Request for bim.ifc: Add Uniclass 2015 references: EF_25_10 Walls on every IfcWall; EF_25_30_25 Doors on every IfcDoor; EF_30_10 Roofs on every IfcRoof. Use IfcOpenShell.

First a look at what the model holds.

```python
import ifcopenshell

model = ifcopenshell.open("bim.ifc")
print(model.schema)
print("classifications:", [c.Name for c in model.by_type("IfcClassification")])
for ifc_class in ("IfcDoor", "IfcRoof", "IfcStair", "IfcWall", "IfcWindow"):
    print(ifc_class, len(model.by_type(ifc_class)))
```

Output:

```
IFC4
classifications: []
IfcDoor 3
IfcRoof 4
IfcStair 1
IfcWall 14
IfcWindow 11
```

```python
import ifcopenshell
import ifcopenshell.api.classification

model = ifcopenshell.open("bim.ifc")

system = ifcopenshell.api.classification.add_classification(model, classification="Uniclass 2015")

codes = {
    "IfcWall": ("EF_25_10", "Walls"),
    "IfcDoor": ("EF_25_30_25", "Doors"),
    "IfcRoof": ("EF_30_10", "Roofs"),
}
for ifc_class, (code, name) in codes.items():
    products = model.by_type(ifc_class)
    ifcopenshell.api.classification.add_reference(
        model, products=products, classification=system, identification=code, name=name
    )
    print(code, len(products))

model.write("bim_v2.ifc")
```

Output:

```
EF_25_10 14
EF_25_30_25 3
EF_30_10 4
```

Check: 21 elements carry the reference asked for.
